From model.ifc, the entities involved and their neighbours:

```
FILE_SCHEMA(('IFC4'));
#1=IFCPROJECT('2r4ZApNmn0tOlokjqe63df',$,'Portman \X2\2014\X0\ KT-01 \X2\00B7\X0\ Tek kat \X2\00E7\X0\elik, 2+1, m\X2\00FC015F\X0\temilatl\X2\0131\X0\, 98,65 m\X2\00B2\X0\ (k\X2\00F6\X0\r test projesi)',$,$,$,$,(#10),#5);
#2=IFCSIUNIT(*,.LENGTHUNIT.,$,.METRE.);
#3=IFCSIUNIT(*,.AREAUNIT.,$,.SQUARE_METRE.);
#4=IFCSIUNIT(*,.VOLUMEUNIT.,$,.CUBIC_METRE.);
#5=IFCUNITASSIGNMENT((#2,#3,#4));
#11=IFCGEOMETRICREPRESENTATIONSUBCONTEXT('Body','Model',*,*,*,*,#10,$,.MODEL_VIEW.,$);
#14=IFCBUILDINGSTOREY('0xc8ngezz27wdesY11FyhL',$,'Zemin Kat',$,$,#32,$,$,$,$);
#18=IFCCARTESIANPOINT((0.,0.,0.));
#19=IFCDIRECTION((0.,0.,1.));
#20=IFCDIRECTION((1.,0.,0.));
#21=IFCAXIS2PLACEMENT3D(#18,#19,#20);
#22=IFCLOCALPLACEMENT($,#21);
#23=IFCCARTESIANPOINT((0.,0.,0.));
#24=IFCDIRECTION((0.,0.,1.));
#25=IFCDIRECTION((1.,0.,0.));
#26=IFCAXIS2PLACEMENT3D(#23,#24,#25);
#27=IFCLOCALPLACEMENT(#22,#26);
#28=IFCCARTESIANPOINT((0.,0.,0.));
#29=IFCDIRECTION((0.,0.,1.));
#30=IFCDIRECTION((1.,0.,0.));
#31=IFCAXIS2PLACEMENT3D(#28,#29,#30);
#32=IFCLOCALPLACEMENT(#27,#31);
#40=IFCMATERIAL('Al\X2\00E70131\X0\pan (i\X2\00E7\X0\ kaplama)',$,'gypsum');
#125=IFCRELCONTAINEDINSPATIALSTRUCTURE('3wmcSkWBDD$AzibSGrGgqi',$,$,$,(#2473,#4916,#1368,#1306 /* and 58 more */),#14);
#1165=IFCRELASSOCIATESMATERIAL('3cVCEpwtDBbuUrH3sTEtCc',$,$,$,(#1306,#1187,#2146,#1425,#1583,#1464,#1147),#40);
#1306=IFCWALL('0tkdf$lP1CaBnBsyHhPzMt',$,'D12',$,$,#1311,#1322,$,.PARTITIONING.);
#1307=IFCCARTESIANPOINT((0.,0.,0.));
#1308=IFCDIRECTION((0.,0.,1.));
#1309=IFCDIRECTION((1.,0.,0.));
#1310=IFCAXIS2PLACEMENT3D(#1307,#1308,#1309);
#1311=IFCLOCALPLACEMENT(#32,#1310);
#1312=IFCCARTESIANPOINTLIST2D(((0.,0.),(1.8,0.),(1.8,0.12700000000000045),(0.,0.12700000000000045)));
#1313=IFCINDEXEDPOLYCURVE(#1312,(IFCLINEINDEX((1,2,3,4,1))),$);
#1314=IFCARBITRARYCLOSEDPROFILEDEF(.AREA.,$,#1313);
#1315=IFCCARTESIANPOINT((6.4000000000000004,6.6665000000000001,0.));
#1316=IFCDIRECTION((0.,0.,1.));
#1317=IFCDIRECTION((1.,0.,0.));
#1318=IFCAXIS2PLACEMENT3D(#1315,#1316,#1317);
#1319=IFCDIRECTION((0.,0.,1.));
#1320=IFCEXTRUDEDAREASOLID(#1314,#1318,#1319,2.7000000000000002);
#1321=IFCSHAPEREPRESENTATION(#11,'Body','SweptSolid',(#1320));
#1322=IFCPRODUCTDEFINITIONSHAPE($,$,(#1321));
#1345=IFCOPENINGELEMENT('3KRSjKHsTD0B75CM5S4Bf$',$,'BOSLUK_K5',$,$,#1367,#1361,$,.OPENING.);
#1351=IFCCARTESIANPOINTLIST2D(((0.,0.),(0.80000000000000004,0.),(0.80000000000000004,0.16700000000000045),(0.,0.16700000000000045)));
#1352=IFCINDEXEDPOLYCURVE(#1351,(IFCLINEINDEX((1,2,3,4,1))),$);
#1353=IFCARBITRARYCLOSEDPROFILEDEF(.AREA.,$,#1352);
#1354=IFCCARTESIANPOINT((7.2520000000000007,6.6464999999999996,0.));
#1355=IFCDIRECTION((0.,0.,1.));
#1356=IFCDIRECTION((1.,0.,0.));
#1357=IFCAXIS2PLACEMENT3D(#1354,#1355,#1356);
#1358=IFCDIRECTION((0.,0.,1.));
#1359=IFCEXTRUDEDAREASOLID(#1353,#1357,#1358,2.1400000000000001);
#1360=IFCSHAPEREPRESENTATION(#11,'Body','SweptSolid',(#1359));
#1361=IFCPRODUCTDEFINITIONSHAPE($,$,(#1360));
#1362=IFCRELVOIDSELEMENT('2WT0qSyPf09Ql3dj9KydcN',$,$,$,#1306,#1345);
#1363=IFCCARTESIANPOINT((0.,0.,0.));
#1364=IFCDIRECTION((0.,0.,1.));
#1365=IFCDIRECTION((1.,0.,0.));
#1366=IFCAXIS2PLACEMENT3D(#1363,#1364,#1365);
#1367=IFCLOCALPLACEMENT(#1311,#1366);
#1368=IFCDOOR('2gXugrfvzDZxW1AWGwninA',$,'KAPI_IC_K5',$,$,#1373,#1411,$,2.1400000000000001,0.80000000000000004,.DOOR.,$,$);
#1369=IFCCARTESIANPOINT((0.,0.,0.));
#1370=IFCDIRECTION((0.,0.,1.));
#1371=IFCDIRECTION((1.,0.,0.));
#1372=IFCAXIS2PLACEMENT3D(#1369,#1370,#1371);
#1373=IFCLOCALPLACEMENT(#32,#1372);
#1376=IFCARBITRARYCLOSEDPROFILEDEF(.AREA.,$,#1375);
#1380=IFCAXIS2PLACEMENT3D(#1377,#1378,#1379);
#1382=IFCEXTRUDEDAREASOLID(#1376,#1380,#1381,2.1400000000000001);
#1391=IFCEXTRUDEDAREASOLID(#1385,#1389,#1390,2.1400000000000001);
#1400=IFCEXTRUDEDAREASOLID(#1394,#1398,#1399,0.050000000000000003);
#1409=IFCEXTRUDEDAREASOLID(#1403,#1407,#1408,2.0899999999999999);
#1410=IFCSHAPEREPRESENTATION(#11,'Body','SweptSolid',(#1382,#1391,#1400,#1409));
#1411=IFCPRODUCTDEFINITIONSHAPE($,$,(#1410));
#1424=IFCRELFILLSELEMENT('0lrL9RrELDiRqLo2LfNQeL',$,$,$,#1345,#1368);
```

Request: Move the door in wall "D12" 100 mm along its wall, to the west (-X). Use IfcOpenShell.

```python
import ifcopenshell
import ifcopenshell.api.geometry
import ifcopenshell.util.placement

model = ifcopenshell.open("model.ifc")

door = model.by_id(1368)
opening = door.FillsVoids[0].RelatingOpeningElement
wall = opening.VoidsElements[0].RelatingBuildingElement

wall_matrix = ifcopenshell.util.placement.get_local_placement(wall.ObjectPlacement)
shift = wall_matrix[:3, 0] * -0.1
before = ifcopenshell.util.placement.get_local_placement(door.ObjectPlacement)[:3, 3].copy()

# The door is not placed relative to its opening, so move both.
for product in (opening, door):
    matrix = ifcopenshell.util.placement.get_local_placement(product.ObjectPlacement)
    matrix[:3, 3] += shift
    ifcopenshell.api.geometry.edit_object_placement(model, product=product, matrix=matrix, is_si=False)

after = ifcopenshell.util.placement.get_local_placement(door.ObjectPlacement)[:3, 3]
print("door moved by", (after - before).round(3) + 0.0)

model.write("model_updated.ifc")
```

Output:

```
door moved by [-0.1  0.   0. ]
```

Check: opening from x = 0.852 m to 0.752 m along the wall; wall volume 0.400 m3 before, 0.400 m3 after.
